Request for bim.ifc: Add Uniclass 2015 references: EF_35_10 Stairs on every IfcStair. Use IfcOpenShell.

First a look at what the model holds.

```python
import ifcopenshell

model = ifcopenshell.open("bim.ifc")
print(model.schema)
print("classifications:", [c.Name for c in model.by_type("IfcClassification")])
for ifc_class in ("IfcDoor", "IfcRoof", "IfcStair", "IfcWall", "IfcWindow"):
    print(ifc_class, len(model.by_type(ifc_class)))
```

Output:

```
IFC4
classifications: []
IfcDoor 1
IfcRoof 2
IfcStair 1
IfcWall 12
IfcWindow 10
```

```python
import ifcopenshell
import ifcopenshell.api.classification

model = ifcopenshell.open("bim.ifc")

system = ifcopenshell.api.classification.add_classification(model, classification="Uniclass 2015")

codes = {
    "IfcStair": ("EF_35_10", "Stairs"),
}
for ifc_class, (code, name) in codes.items():
    products = model.by_type(ifc_class)
    ifcopenshell.api.classification.add_reference(
        model, products=products, classification=system, identification=code, name=name
    )
    print(code, len(products))

model.write("bim_v2.ifc")
```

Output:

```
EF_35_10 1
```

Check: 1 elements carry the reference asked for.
